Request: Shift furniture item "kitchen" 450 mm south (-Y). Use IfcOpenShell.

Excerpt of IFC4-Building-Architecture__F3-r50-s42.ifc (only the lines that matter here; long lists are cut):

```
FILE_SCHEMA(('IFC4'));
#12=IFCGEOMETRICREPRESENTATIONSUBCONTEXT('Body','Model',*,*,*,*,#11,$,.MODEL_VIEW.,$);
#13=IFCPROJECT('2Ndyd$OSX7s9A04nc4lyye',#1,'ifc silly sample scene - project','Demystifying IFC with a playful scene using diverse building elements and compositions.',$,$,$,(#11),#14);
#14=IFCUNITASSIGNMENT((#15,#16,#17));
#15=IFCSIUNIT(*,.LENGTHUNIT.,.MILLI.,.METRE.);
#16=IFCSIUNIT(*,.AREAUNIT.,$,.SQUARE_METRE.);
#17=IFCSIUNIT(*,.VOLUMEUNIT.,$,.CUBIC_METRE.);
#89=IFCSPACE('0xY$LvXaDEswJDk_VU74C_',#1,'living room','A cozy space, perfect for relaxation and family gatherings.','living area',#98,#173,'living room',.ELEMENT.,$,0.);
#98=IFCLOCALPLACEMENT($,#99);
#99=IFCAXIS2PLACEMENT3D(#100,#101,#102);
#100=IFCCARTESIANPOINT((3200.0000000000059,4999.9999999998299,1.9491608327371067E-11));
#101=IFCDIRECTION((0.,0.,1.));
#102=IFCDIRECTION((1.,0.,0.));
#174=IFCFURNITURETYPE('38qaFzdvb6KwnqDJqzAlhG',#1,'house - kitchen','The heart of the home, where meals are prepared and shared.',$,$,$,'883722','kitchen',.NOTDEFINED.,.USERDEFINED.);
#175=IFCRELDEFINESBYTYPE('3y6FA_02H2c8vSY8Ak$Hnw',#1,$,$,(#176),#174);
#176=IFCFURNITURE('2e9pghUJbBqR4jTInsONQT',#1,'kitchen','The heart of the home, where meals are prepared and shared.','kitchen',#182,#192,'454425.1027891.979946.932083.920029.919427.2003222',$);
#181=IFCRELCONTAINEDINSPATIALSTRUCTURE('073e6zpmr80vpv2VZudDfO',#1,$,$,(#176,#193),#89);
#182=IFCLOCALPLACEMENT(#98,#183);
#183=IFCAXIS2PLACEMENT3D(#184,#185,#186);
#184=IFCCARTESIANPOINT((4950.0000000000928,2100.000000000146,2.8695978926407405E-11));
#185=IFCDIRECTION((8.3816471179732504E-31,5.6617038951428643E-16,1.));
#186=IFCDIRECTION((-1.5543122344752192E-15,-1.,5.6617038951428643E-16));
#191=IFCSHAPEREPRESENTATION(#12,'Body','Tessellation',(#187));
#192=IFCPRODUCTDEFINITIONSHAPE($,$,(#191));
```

```python
import ifcopenshell
import ifcopenshell.api.geometry
import ifcopenshell.util.placement

model = ifcopenshell.open("IFC4-Building-Architecture__F3-r50-s42.ifc")

item = model.by_guid("2e9pghUJbBqR4jTInsONQT")
matrix = ifcopenshell.util.placement.get_local_placement(item.ObjectPlacement)
matrix[1, 3] -= 450.0
ifcopenshell.api.geometry.edit_object_placement(model, product=item, matrix=matrix, is_si=False)

print(ifcopenshell.util.placement.get_local_placement(item.ObjectPlacement).round(3) + 0.0)

model.write("IFC4-Building-Architecture__F3-r50-s42_edited.ifc")
```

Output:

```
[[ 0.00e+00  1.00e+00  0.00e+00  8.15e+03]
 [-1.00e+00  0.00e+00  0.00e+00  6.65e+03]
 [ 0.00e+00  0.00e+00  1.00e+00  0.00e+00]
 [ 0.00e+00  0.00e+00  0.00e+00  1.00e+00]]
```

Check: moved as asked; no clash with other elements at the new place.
